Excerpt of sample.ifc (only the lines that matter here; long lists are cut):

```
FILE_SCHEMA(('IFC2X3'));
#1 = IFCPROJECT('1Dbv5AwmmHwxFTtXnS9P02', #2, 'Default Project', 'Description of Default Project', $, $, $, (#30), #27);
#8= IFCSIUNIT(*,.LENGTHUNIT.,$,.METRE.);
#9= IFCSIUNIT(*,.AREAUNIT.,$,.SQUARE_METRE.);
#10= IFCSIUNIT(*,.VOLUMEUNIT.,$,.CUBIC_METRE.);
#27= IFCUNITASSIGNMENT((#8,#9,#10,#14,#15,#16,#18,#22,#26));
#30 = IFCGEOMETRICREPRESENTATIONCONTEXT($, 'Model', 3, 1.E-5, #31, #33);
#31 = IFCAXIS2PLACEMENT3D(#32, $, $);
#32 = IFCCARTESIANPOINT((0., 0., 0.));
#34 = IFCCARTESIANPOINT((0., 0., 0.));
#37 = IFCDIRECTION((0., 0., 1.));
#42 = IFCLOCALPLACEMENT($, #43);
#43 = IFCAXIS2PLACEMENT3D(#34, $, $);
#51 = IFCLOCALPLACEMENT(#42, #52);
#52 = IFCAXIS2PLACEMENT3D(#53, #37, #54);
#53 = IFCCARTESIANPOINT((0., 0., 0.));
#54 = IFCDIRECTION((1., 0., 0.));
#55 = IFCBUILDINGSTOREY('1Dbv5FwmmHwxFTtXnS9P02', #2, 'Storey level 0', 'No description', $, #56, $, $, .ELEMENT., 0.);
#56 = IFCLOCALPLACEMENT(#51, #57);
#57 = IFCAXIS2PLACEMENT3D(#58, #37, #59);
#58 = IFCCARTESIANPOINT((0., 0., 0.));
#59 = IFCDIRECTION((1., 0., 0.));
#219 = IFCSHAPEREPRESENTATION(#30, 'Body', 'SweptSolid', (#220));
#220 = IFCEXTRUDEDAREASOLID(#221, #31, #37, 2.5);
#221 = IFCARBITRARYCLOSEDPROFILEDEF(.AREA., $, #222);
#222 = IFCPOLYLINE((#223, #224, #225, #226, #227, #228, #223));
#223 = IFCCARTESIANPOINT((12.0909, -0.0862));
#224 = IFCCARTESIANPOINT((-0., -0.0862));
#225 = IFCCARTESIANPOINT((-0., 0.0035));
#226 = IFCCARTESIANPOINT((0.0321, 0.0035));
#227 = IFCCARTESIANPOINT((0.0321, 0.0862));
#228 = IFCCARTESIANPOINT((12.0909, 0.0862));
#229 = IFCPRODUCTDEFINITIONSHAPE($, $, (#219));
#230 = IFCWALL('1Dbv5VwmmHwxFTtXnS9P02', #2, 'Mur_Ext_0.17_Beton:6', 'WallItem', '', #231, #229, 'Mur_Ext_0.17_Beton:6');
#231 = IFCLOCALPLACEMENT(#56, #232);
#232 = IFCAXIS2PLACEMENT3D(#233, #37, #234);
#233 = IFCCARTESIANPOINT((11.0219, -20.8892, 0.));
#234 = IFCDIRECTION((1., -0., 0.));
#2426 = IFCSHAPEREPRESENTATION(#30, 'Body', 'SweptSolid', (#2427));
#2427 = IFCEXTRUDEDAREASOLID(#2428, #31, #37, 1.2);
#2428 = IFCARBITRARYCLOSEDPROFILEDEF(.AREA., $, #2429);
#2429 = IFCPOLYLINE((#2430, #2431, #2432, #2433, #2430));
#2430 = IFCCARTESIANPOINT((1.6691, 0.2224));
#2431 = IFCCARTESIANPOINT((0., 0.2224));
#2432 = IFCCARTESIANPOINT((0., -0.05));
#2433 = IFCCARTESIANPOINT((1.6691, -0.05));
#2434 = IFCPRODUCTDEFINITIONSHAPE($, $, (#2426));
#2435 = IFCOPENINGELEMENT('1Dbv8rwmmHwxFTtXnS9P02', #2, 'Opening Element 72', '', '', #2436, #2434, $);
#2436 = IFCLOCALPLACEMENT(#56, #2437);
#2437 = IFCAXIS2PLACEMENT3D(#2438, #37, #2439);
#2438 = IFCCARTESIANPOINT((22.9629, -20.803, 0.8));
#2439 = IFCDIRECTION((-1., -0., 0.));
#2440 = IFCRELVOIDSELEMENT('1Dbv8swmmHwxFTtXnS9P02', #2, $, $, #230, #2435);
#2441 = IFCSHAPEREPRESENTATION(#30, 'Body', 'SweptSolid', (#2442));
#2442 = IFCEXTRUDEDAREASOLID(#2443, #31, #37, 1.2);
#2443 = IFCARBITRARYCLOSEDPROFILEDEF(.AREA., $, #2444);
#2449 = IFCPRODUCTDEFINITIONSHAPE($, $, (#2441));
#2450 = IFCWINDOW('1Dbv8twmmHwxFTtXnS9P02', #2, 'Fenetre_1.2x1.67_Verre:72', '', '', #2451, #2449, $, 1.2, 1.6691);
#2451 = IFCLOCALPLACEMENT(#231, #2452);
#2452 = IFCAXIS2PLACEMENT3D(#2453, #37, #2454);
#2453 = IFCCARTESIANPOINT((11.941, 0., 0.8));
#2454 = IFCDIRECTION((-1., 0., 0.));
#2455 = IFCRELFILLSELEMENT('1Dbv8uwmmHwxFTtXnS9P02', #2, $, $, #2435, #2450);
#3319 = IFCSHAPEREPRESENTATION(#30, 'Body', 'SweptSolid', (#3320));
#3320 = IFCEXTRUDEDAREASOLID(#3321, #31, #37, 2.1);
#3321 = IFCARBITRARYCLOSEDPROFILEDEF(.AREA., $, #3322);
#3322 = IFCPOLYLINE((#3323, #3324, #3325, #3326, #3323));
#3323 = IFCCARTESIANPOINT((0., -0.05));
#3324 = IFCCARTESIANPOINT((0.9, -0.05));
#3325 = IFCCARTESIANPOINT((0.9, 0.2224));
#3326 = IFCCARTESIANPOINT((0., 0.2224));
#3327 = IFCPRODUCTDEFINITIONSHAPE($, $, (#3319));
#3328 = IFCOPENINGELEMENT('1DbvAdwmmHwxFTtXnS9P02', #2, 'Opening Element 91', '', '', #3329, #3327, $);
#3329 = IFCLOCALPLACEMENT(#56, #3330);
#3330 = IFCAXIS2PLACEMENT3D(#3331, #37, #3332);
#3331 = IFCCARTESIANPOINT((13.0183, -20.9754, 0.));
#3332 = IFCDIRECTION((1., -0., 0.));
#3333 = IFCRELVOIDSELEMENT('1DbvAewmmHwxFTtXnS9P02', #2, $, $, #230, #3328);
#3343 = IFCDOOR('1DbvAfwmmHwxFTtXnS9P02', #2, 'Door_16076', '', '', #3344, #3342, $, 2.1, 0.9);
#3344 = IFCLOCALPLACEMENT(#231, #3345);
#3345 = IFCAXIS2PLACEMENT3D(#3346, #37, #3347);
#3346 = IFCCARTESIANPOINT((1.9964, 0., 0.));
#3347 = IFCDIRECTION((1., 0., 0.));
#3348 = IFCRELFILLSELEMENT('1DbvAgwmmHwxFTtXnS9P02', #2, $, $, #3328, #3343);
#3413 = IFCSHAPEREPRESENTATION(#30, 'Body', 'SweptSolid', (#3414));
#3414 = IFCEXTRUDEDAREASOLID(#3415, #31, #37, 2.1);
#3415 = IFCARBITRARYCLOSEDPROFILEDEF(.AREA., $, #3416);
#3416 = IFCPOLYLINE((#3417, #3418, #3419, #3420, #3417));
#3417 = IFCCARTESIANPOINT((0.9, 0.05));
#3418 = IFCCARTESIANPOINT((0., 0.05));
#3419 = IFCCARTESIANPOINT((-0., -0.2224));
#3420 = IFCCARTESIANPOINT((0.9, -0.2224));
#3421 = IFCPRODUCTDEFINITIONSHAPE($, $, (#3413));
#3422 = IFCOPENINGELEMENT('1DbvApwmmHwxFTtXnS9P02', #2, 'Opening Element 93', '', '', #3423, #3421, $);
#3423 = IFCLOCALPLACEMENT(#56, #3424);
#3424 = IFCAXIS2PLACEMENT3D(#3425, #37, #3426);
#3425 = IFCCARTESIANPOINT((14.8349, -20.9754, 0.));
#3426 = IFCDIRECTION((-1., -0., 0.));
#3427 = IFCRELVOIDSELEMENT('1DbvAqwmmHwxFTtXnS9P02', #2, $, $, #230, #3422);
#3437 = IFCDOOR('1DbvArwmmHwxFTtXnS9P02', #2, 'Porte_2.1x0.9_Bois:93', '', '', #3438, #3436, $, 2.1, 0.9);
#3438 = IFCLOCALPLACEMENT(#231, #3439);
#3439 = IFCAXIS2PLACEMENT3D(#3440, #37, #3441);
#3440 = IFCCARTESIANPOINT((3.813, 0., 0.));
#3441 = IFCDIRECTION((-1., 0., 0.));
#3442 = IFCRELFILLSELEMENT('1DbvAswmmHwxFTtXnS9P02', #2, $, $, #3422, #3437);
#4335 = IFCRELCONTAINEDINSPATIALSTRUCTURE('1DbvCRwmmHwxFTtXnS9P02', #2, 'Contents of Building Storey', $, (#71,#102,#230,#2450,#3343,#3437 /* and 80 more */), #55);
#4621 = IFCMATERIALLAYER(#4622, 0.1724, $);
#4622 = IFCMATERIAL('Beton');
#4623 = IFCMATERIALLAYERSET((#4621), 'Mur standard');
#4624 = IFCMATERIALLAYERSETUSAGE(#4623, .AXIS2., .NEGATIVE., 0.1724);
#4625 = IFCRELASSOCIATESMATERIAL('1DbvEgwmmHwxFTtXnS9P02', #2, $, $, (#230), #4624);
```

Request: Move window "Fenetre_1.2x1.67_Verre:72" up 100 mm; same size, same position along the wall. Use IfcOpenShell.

```python
import numpy as np
import ifcopenshell
import ifcopenshell.api.geometry
import ifcopenshell.util.placement
import ifcopenshell.util.unit

model = ifcopenshell.open("sample.ifc")
unit_scale = ifcopenshell.util.unit.calculate_unit_scale(model)

window = model.by_guid("1Dbv8twmmHwxFTtXnS9P02")
opening = window.FillsVoids[0].RelatingOpeningElement
dz = 0.1

shift = np.array([0.0, 0.0, dz])
# The window is not placed relative to its opening, so move both.
for product in (opening, window):
    matrix = ifcopenshell.util.placement.get_local_placement(product.ObjectPlacement)
    matrix[:3, 3] += shift
    ifcopenshell.api.geometry.edit_object_placement(model, product=product, matrix=matrix, is_si=False)

print(f"moved by {dz * unit_scale:+.3f} m")

model.write("sample_updated.ifc")
```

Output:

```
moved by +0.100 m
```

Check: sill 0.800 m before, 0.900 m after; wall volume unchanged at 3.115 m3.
